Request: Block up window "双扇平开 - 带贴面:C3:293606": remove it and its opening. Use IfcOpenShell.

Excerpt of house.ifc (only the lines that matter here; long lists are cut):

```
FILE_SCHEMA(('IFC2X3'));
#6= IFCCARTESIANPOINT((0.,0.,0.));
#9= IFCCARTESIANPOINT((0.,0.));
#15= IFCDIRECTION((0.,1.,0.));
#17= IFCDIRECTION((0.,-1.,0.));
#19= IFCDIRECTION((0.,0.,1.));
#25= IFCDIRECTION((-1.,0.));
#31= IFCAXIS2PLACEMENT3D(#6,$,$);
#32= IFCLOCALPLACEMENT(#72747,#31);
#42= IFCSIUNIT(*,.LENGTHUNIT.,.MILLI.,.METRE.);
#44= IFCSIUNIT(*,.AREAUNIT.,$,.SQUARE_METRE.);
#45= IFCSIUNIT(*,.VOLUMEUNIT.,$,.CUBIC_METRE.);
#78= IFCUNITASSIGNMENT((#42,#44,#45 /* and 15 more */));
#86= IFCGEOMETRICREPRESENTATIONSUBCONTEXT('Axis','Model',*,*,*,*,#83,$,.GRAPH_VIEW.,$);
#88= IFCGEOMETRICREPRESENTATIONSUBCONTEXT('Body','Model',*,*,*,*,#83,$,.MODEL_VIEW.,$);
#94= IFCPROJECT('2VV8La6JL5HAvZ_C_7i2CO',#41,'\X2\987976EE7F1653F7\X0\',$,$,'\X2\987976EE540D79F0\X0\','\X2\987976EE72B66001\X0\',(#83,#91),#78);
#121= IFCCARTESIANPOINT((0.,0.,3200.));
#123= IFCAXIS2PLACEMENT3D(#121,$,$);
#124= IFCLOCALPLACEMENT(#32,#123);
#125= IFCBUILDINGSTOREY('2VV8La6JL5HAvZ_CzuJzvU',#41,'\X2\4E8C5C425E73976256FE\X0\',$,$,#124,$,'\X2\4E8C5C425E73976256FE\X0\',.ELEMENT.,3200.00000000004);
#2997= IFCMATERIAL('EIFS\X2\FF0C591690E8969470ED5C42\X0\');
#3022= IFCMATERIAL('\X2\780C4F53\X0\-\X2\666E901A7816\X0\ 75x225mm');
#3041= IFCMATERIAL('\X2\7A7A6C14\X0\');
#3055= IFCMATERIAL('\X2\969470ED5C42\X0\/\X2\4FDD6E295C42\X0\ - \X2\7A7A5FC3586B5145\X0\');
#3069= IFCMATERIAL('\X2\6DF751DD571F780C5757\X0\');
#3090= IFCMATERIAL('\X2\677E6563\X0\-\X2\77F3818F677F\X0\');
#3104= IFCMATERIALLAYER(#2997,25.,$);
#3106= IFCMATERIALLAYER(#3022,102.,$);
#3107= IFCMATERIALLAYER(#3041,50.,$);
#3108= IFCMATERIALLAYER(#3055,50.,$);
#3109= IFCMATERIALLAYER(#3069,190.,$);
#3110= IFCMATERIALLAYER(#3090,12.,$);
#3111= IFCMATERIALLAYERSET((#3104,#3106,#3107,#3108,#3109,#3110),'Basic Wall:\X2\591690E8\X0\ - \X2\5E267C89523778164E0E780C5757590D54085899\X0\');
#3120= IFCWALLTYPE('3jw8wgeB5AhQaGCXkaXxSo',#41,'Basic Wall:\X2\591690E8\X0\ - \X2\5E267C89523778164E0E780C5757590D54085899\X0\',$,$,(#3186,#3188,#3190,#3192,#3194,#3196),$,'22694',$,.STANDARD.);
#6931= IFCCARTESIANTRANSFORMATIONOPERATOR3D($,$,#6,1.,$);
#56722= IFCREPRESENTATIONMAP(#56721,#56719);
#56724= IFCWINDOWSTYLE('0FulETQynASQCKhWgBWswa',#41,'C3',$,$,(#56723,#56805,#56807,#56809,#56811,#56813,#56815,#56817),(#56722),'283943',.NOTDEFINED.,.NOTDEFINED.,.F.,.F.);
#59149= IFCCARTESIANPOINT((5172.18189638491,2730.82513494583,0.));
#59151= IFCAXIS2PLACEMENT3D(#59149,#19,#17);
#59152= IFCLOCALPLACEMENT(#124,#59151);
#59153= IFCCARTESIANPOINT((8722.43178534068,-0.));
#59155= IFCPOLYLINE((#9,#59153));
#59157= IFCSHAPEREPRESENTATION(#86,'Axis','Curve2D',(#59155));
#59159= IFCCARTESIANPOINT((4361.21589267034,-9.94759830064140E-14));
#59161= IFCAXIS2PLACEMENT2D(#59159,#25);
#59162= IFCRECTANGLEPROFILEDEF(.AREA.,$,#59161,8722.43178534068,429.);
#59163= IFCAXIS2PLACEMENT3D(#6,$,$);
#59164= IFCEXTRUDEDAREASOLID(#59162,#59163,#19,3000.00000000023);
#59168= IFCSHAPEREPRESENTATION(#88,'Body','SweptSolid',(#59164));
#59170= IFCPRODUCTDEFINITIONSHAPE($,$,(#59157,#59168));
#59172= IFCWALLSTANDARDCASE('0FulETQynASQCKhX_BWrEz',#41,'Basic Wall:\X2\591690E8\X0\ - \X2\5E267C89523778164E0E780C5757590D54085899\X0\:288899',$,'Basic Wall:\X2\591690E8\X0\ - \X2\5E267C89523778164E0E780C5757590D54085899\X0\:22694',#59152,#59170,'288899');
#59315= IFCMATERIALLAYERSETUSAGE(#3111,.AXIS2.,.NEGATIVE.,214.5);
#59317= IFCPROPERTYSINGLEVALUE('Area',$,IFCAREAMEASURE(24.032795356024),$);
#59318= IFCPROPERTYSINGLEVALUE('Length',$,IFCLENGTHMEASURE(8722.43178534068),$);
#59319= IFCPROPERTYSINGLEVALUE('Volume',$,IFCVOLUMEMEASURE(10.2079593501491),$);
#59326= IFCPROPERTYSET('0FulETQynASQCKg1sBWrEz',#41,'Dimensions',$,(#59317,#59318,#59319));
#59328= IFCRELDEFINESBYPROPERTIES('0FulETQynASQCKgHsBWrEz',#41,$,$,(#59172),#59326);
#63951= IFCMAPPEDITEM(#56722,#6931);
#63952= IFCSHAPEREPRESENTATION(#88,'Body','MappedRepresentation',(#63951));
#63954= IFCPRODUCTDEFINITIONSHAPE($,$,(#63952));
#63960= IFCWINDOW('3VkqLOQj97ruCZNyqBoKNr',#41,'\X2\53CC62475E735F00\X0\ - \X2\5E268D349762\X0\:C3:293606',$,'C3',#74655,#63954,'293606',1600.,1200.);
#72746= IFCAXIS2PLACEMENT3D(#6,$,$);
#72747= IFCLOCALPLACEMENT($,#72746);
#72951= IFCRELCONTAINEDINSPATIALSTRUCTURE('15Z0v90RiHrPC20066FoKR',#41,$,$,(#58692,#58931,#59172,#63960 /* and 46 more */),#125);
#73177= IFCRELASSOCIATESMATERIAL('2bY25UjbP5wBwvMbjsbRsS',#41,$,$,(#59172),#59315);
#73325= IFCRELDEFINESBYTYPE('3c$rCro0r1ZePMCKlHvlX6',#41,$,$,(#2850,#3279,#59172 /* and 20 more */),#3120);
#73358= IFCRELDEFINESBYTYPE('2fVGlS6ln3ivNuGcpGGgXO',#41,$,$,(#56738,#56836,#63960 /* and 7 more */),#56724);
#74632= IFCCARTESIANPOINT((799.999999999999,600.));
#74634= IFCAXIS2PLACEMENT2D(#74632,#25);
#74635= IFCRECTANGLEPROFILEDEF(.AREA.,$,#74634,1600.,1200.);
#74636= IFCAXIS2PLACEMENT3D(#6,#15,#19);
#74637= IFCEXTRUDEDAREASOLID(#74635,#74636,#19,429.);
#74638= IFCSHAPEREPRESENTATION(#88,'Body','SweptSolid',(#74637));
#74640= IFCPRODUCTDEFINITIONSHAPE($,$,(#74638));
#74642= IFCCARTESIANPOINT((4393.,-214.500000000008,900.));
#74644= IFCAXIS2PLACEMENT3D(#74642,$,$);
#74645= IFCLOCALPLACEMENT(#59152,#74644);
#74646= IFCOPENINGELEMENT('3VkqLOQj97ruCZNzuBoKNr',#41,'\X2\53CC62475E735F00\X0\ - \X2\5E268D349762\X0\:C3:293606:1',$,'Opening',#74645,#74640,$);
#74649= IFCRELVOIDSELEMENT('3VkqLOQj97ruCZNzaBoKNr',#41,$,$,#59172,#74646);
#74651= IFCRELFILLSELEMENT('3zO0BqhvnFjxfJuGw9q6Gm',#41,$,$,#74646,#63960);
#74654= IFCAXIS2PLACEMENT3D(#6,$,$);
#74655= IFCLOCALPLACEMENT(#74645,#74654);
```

```python
import ifcopenshell
import ifcopenshell.api.feature
import ifcopenshell.api.pset
import ifcopenshell.api.root
import ifcopenshell.geom
import ifcopenshell.util.element
import ifcopenshell.util.shape
import ifcopenshell.util.unit

model = ifcopenshell.open("house.ifc")
area_scale = ifcopenshell.util.unit.calculate_unit_scale(model, "AREAUNIT")
volume_scale = ifcopenshell.util.unit.calculate_unit_scale(model, "VOLUMEUNIT")
settings = ifcopenshell.geom.settings()


def volume(element):
    """Net volume in cubic metres, openings subtracted."""
    shape = ifcopenshell.geom.create_shape(settings, element)
    return ifcopenshell.util.shape.get_volume(shape.geometry)


window = model.by_guid("3VkqLOQj97ruCZNyqBoKNr")
opening = window.FillsVoids[0].RelatingOpeningElement
wall = opening.VoidsElements[0].RelatingBuildingElement
before = volume(wall)

ifcopenshell.api.root.remove_product(model, product=window)
ifcopenshell.api.feature.remove_feature(model, feature=opening)

after = volume(wall)
thickness = 0.429  # wall thickness in metres

# Update the wall's stored quantities.
pset = model.by_id(ifcopenshell.util.element.get_pset(wall, "Dimensions", should_inherit=False)["id"])
ifcopenshell.api.pset.edit_pset(model, pset=pset, properties={
    "Area": model.create_entity("IfcAreaMeasure", after / thickness / area_scale),
    "Volume": model.create_entity("IfcVolumeMeasure", after / volume_scale),
})

print(f"wall volume {before:.3f} -> {after:.3f} m3")

model.write("house_updated.ifc")
```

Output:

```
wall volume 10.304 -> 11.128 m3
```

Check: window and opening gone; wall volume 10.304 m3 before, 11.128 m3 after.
